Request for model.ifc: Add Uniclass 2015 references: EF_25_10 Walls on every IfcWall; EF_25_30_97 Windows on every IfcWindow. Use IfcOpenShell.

First a look at what the model holds.

```python
import ifcopenshell

model = ifcopenshell.open("model.ifc")
print(model.schema)
print("classifications:", [c.Name for c in model.by_type("IfcClassification")])
for ifc_class in ("IfcDoor", "IfcRoof", "IfcStair", "IfcWall", "IfcWindow"):
    print(ifc_class, len(model.by_type(ifc_class)))
```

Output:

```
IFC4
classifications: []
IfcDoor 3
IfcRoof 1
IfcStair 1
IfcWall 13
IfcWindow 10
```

```python
import ifcopenshell
import ifcopenshell.api.classification

model = ifcopenshell.open("model.ifc")

system = ifcopenshell.api.classification.add_classification(model, classification="Uniclass 2015")

codes = {
    "IfcWall": ("EF_25_10", "Walls"),
    "IfcWindow": ("EF_25_30_97", "Windows"),
}
for ifc_class, (code, name) in codes.items():
    products = model.by_type(ifc_class)
    ifcopenshell.api.classification.add_reference(
        model, products=products, classification=system, identification=code, name=name
    )
    print(code, len(products))

model.write("model_v2.ifc")
```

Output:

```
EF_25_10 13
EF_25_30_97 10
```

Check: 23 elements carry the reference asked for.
